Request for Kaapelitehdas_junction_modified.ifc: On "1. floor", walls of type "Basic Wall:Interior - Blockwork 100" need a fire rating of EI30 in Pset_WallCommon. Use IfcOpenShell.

First a look at what the model holds.

```python
import ifcopenshell
import ifcopenshell.util.element

model = ifcopenshell.open("Kaapelitehdas_junction_modified.ifc")
print(model.schema)
storey = next(s for s in model.by_type("IfcBuildingStorey") if s.Name == "1. floor")
walls = [e for e in ifcopenshell.util.element.get_decomposition(storey) if e.is_a("IfcWall")]
seen = {}
for e in walls:
    element_type = ifcopenshell.util.element.get_type(e)
    key = (element_type.Name if element_type != e and element_type else None, ifcopenshell.util.element.get_pset(e, "Pset_WallCommon", "FireRating"))
    seen[key] = seen.get(key, 0) + 1
for (name, value), count in sorted(seen.items(), key=str):
    print(count, "x", name, "|", value)
```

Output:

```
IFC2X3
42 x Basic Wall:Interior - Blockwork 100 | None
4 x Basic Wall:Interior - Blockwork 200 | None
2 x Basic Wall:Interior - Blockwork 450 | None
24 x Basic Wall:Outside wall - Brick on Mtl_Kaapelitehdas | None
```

```python
import ifcopenshell
import ifcopenshell.api.pset
import ifcopenshell.util.element

model = ifcopenshell.open("Kaapelitehdas_junction_modified.ifc")

storey = next(s for s in model.by_type("IfcBuildingStorey") if s.Name == "1. floor")
walls = [e for e in ifcopenshell.util.element.get_decomposition(storey) if e.is_a("IfcWall")]

count = 0
for e in walls:
    element_type = ifcopenshell.util.element.get_type(e)
    if element_type in (None, e) or element_type.Name != "Basic Wall:Interior - Blockwork 100":
        continue
    # add_pset returns the element's existing set when there is one.
    pset = ifcopenshell.api.pset.add_pset(model, product=e, name="Pset_WallCommon")
    ifcopenshell.api.pset.edit_pset(model, pset=pset, properties={"FireRating": "EI30"})
    count += 1

print(count, "walls updated")

model.write("Kaapelitehdas_junction_modified_v2.ifc")
```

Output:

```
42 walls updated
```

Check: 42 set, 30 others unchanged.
